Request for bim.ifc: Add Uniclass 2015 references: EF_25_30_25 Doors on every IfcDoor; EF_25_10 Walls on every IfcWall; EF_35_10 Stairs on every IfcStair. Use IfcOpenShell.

First a look at what the model holds.

```python
import ifcopenshell

model = ifcopenshell.open("bim.ifc")
print(model.schema)
print("classifications:", [c.Name for c in model.by_type("IfcClassification")])
for ifc_class in ("IfcDoor", "IfcRoof", "IfcStair", "IfcWall", "IfcWindow"):
    print(ifc_class, len(model.by_type(ifc_class)))
```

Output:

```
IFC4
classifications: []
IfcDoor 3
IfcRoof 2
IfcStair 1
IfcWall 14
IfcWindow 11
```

```python
import ifcopenshell
import ifcopenshell.api.classification

model = ifcopenshell.open("bim.ifc")

system = ifcopenshell.api.classification.add_classification(model, classification="Uniclass 2015")

codes = {
    "IfcDoor": ("EF_25_30_25", "Doors"),
    "IfcWall": ("EF_25_10", "Walls"),
    "IfcStair": ("EF_35_10", "Stairs"),
}
for ifc_class, (code, name) in codes.items():
    products = model.by_type(ifc_class)
    ifcopenshell.api.classification.add_reference(
        model, products=products, classification=system, identification=code, name=name
    )
    print(code, len(products))

model.write("bim-out.ifc")
```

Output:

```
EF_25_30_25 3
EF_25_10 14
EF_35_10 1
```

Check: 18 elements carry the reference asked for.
